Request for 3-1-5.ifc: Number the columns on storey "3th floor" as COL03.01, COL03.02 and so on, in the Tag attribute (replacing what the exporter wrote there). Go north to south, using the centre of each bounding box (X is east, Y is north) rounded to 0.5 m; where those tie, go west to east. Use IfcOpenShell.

First a look at what the model holds.

```python
import ifcopenshell
import ifcopenshell.util.element
import ifcopenshell.util.placement

model = ifcopenshell.open("3-1-5.ifc")
print(model.schema)
storey = next(s for s in model.by_type("IfcBuildingStorey") if s.Name == "3th floor")
columns = [e for e in ifcopenshell.util.element.get_decomposition(storey) if e.is_a("IfcColumn")]
for e in sorted(columns, key=lambda e: e.id()):
    origin = ifcopenshell.util.placement.get_local_placement(e.ObjectPlacement)[:3, 3]
    print(e.id(), e.Tag, e.Name, origin.round(2) + 0.0, sep=" | ")
```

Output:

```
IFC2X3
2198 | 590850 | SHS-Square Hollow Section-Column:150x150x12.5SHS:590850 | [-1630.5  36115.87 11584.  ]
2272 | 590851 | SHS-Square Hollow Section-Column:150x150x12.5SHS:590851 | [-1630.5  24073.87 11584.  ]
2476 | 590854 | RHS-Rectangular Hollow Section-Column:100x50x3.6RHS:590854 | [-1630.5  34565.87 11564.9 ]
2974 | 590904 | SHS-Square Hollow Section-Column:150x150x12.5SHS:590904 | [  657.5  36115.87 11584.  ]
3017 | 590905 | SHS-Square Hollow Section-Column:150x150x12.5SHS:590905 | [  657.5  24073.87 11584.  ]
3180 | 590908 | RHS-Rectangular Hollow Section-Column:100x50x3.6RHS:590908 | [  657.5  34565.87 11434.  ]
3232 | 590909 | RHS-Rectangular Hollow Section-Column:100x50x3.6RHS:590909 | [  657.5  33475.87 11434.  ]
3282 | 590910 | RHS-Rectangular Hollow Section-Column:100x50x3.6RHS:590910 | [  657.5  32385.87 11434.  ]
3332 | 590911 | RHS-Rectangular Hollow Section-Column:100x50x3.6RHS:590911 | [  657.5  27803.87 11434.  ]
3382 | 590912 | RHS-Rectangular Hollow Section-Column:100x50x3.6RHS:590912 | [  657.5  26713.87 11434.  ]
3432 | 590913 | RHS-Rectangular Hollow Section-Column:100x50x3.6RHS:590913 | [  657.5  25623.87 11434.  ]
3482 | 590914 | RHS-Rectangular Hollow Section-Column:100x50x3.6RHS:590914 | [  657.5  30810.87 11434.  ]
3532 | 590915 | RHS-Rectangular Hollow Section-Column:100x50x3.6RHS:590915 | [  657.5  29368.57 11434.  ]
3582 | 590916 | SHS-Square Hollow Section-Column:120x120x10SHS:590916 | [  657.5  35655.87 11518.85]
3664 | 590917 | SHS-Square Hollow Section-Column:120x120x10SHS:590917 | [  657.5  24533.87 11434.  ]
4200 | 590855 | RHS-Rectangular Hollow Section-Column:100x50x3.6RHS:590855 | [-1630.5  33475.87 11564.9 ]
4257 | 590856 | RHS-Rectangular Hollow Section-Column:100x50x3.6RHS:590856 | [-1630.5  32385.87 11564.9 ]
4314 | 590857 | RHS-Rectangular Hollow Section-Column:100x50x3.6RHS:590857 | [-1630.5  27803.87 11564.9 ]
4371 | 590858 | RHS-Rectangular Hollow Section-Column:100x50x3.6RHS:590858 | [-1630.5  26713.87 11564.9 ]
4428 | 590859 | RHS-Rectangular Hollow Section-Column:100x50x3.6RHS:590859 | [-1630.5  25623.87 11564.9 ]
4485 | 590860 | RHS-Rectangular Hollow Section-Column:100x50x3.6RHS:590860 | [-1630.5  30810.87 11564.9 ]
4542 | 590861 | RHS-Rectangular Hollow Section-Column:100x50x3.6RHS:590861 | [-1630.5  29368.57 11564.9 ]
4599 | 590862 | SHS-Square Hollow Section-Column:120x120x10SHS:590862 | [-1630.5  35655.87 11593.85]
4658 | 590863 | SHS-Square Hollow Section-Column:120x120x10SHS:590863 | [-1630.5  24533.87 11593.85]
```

```python
import ifcopenshell
import ifcopenshell.geom
import ifcopenshell.util.element
import ifcopenshell.util.shape

model = ifcopenshell.open("3-1-5.ifc")
settings = ifcopenshell.geom.settings()
settings.set("use-world-coords", True)


def centre(element):
    shape = ifcopenshell.geom.create_shape(settings, element)
    return ifcopenshell.util.shape.get_bbox_centroid(shape.geometry)


storey = next(s for s in model.by_type("IfcBuildingStorey") if s.Name == "3th floor")
columns = [e for e in ifcopenshell.util.element.get_decomposition(storey) if e.is_a("IfcColumn")]

# Insertion points can sit at a corner or the storey origin, so sort by the geometry (in metres).
centres = {e: centre(e) for e in columns}
columns.sort(key=lambda e: (-round(centres[e][1] / 0.5), centres[e][0]))

for i, e in enumerate(columns, start=1):
    number = f"COL03.{i:02d}"
    e.Tag = number
    print(e.id(), number)

model.write("3-1-5_updated.ifc")
```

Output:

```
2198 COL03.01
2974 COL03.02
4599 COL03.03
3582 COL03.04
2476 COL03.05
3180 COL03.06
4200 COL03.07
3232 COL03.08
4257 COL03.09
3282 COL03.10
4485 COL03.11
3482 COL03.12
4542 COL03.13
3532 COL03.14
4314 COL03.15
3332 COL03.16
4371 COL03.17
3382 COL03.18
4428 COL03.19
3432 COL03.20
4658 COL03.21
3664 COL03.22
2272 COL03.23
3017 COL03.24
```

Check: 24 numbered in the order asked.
